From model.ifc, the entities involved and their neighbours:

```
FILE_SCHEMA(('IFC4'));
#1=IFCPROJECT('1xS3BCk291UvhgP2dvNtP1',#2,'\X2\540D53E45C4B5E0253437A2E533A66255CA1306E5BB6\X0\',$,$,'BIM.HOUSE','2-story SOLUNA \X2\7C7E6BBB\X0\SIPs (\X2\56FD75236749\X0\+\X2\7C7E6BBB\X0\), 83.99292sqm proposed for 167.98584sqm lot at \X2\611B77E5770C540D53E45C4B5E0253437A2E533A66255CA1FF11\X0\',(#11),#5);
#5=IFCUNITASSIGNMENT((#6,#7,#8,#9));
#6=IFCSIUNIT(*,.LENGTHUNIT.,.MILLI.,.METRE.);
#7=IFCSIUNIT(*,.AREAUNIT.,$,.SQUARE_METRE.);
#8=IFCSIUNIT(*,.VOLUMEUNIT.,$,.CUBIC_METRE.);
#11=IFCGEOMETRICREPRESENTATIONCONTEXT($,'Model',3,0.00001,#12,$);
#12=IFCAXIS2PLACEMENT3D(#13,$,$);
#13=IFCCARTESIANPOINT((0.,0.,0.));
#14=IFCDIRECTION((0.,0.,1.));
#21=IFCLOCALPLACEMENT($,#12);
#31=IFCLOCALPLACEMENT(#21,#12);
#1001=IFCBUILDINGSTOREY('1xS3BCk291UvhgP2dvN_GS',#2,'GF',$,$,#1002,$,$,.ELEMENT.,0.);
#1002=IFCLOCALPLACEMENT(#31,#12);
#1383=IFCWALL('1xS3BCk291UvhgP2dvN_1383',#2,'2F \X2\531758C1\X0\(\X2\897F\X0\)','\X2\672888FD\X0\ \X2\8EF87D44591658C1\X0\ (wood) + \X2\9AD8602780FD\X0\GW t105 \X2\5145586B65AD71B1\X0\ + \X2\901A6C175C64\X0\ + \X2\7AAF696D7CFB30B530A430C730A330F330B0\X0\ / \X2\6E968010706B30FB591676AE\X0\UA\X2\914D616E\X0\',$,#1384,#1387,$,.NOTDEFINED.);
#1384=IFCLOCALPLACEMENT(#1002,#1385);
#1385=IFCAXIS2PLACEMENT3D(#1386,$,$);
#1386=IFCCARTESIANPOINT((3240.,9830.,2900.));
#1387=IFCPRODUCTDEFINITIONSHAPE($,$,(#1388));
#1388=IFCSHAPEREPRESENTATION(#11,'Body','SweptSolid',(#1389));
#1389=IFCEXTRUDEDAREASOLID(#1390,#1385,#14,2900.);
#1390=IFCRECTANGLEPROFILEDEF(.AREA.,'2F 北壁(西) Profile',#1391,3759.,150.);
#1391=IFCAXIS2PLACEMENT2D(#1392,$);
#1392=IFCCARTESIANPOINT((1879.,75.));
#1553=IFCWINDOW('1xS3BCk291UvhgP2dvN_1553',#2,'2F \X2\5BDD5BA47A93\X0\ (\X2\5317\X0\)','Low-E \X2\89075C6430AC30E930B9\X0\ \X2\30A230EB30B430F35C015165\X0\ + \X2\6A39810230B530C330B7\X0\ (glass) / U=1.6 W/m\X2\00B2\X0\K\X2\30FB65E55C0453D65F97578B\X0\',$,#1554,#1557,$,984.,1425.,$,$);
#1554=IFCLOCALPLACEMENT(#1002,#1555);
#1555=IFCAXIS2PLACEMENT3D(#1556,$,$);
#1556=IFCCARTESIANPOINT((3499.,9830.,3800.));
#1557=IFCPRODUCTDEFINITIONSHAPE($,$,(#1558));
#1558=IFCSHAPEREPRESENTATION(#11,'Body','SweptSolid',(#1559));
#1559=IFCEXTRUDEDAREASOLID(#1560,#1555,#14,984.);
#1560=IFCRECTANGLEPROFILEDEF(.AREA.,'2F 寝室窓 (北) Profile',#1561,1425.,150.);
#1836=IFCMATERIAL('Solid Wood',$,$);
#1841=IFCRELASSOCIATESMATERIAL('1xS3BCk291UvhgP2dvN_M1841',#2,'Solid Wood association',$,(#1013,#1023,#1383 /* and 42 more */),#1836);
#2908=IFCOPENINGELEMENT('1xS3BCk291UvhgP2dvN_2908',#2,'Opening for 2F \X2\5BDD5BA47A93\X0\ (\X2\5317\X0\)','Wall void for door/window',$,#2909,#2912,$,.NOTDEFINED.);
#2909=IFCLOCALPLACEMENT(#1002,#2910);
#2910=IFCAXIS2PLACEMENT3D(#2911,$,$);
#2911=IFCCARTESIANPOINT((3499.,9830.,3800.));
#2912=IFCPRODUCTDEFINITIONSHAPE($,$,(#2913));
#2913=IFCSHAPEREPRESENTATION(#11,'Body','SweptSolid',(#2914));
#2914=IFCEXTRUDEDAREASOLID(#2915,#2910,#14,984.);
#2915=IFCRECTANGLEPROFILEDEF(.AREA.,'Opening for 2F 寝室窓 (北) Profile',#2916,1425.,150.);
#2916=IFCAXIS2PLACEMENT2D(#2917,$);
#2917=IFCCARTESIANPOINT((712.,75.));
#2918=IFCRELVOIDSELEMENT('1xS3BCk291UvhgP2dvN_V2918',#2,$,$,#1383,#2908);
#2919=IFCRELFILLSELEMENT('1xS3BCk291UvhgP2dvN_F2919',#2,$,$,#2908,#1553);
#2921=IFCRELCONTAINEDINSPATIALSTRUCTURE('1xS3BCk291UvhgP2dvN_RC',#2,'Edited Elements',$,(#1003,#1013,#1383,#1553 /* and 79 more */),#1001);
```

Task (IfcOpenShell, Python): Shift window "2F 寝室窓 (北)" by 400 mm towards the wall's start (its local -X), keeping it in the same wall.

```python
import ifcopenshell
import ifcopenshell.api.geometry
import ifcopenshell.util.placement
import ifcopenshell.util.unit

model = ifcopenshell.open("model.ifc")
unit_scale = ifcopenshell.util.unit.calculate_unit_scale(model)

window = model.by_guid("1xS3BCk291UvhgP2dvN_1553")
opening = window.FillsVoids[0].RelatingOpeningElement
wall = opening.VoidsElements[0].RelatingBuildingElement

wall_matrix = ifcopenshell.util.placement.get_local_placement(wall.ObjectPlacement)
shift = wall_matrix[:3, 0] * -0.4 / unit_scale
before = ifcopenshell.util.placement.get_local_placement(window.ObjectPlacement)[:3, 3].copy()

# The window is not placed relative to its opening, so move both.
for product in (opening, window):
    matrix = ifcopenshell.util.placement.get_local_placement(product.ObjectPlacement)
    matrix[:3, 3] += shift
    ifcopenshell.api.geometry.edit_object_placement(model, product=product, matrix=matrix, is_si=False)

after = ifcopenshell.util.placement.get_local_placement(window.ObjectPlacement)[:3, 3]
print("window moved by", (after - before).round(3) + 0.0)

model.write("model_rev.ifc")
```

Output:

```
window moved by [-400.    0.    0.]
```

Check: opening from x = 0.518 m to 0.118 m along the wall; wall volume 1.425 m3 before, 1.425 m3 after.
